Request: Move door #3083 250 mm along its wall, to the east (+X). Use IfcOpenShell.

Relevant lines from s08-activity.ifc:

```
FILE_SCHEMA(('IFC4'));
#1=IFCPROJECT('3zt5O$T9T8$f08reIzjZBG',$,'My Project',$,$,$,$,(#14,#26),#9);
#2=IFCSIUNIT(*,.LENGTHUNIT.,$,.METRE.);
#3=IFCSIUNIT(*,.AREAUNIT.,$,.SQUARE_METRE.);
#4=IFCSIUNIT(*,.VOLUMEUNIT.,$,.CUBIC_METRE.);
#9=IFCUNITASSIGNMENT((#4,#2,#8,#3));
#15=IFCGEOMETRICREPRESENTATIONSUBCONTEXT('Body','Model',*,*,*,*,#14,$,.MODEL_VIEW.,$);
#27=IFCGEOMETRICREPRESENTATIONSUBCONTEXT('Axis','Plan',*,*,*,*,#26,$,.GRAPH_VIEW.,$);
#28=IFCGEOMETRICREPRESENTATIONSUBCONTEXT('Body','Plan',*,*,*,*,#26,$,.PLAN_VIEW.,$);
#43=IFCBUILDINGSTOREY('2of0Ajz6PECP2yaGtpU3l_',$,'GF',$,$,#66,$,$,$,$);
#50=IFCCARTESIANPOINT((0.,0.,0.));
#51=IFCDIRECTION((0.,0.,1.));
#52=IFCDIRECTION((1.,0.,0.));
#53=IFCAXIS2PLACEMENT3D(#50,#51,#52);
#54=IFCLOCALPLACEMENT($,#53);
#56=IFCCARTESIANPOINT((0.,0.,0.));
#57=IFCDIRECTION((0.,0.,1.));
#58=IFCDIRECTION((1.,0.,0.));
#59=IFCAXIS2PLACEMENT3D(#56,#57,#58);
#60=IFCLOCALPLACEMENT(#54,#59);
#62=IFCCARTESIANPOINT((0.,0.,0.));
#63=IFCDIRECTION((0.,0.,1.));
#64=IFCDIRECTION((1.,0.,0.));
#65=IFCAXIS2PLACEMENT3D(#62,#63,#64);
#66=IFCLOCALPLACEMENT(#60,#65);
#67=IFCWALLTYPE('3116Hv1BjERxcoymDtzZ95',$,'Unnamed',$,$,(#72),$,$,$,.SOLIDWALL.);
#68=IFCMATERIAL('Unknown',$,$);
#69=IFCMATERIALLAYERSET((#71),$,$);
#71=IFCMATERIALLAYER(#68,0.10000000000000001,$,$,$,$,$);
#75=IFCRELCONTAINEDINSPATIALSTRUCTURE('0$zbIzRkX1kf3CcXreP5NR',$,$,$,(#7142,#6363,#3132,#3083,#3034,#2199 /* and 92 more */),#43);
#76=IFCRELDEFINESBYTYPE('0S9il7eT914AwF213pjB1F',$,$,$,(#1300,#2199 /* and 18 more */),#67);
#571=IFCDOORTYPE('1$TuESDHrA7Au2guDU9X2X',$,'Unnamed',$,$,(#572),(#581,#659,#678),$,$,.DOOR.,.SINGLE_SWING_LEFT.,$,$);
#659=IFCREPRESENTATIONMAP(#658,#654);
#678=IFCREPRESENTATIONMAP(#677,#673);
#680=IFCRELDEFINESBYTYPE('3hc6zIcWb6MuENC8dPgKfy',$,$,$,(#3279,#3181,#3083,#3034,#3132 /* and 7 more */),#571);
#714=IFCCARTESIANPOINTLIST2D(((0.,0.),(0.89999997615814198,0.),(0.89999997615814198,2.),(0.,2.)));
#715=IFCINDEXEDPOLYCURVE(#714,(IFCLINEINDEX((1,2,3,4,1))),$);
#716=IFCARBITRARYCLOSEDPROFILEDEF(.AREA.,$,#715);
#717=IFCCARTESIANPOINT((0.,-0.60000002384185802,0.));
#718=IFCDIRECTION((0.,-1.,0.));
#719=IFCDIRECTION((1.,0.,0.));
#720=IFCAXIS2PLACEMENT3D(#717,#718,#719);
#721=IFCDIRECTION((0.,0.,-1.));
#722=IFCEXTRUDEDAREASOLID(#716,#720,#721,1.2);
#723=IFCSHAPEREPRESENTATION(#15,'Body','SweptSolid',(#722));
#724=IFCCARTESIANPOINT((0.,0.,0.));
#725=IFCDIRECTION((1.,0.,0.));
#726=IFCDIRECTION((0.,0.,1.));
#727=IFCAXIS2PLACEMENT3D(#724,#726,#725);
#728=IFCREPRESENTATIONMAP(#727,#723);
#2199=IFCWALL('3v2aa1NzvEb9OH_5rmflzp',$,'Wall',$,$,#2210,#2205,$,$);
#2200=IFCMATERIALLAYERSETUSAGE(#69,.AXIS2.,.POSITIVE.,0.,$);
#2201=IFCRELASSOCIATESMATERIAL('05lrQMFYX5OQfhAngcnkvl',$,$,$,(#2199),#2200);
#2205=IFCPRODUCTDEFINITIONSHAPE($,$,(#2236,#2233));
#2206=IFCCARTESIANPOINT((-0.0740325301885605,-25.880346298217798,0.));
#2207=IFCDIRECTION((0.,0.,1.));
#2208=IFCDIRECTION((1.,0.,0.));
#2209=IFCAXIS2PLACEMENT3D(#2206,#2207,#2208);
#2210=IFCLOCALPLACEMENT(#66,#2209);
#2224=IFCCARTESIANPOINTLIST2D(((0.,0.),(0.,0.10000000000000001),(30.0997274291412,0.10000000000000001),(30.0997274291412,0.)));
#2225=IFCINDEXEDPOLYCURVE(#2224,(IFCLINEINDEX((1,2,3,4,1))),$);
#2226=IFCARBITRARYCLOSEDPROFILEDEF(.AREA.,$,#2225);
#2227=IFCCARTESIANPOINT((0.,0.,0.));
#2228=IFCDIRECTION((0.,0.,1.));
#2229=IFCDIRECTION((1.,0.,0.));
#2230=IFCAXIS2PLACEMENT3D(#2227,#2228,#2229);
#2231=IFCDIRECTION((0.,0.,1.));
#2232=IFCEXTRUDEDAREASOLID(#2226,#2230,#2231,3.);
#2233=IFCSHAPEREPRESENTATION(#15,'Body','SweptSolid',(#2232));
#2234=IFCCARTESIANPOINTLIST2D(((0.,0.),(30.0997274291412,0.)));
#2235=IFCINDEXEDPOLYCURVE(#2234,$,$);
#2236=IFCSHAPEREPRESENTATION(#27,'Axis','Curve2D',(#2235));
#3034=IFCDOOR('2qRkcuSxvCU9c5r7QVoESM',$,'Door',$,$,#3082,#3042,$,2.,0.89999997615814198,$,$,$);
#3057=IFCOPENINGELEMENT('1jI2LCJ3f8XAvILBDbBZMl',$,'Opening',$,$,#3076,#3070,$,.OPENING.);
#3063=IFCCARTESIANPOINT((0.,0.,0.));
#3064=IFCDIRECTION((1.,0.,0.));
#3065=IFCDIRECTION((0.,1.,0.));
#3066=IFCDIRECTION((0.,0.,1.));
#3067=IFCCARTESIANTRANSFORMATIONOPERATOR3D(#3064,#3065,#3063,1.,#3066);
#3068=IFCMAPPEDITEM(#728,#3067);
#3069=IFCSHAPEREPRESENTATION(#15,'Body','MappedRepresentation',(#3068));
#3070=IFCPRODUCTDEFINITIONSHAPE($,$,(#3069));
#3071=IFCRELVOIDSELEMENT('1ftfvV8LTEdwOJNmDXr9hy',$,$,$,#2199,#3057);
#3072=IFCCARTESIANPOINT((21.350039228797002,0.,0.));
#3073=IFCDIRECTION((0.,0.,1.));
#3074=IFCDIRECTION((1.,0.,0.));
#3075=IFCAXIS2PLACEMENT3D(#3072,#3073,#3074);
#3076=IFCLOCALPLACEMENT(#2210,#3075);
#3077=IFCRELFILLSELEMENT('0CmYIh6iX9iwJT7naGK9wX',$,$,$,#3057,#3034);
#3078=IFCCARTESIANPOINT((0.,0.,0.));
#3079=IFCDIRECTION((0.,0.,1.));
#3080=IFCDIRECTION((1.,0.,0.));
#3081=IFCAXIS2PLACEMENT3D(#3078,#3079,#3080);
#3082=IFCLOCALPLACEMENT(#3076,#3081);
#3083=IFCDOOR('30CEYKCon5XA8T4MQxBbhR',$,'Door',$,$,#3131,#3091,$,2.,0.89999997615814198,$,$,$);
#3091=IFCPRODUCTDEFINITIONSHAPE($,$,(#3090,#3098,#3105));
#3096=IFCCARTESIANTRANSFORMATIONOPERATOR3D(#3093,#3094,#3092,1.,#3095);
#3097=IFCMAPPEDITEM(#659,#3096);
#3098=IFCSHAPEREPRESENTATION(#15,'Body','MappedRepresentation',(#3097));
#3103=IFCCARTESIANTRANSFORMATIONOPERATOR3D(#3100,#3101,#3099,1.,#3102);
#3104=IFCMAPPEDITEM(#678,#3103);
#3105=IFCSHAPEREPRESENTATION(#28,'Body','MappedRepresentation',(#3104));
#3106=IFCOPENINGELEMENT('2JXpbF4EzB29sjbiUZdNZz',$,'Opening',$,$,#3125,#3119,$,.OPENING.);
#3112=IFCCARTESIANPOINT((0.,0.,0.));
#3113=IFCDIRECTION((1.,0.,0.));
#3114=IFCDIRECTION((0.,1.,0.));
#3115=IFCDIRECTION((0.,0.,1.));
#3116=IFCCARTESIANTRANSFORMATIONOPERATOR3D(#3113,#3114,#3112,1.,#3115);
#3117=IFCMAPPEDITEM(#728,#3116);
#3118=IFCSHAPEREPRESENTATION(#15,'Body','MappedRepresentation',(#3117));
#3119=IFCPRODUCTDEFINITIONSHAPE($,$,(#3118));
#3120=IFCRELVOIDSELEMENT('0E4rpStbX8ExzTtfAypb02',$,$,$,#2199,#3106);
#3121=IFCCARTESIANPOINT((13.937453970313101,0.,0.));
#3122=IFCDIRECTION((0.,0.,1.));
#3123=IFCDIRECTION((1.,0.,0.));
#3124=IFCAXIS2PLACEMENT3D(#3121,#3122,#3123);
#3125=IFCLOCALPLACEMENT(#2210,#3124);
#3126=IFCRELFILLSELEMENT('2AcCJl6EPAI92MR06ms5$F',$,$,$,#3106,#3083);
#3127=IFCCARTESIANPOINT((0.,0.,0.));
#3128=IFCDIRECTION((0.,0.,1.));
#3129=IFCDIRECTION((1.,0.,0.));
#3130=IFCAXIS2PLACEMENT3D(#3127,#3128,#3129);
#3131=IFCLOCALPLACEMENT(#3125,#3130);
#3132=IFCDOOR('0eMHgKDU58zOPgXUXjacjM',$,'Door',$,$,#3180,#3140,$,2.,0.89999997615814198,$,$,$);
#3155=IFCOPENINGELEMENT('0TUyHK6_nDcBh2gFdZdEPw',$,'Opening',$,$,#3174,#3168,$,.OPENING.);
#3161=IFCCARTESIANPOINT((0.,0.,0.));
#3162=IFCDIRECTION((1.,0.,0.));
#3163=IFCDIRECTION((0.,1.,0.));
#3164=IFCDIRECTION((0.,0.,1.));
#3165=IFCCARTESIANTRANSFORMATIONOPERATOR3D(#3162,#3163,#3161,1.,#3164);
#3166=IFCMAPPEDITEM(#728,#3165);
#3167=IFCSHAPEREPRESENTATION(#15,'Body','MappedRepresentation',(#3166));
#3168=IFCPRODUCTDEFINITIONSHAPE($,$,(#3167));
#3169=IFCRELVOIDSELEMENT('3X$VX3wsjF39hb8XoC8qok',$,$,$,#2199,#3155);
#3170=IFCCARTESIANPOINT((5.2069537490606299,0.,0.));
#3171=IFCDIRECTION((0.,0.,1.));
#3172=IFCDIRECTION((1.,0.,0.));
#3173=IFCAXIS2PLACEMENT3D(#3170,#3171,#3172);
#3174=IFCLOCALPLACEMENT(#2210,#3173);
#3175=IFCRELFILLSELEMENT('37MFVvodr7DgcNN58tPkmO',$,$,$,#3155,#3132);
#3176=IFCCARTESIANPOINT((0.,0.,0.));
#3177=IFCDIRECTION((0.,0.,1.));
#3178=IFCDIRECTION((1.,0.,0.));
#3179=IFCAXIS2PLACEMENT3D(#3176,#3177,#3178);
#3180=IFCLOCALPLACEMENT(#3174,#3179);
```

```python
import ifcopenshell
import ifcopenshell.api.geometry
import ifcopenshell.util.placement
import ifcopenshell.util.unit

model = ifcopenshell.open("s08-activity.ifc")
unit_scale = ifcopenshell.util.unit.calculate_unit_scale(model)

door = model.by_guid("30CEYKCon5XA8T4MQxBbhR")
opening = door.FillsVoids[0].RelatingOpeningElement
wall = opening.VoidsElements[0].RelatingBuildingElement

wall_matrix = ifcopenshell.util.placement.get_local_placement(wall.ObjectPlacement)
shift = wall_matrix[:3, 0] * 0.25 / unit_scale
before = ifcopenshell.util.placement.get_local_placement(door.ObjectPlacement)[:3, 3].copy()

# The door is placed relative to its opening, so it follows when the opening moves.
matrix = ifcopenshell.util.placement.get_local_placement(opening.ObjectPlacement)
matrix[:3, 3] += shift
ifcopenshell.api.geometry.edit_object_placement(
    model, product=opening, matrix=matrix, is_si=False, should_transform_children=True
)

after = ifcopenshell.util.placement.get_local_placement(door.ObjectPlacement)[:3, 3]
print("door moved by", (after - before).round(3) + 0.0)

model.write("s08-activity_rev.ifc")
```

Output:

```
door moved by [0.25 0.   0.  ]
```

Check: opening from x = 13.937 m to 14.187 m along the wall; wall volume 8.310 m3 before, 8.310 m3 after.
